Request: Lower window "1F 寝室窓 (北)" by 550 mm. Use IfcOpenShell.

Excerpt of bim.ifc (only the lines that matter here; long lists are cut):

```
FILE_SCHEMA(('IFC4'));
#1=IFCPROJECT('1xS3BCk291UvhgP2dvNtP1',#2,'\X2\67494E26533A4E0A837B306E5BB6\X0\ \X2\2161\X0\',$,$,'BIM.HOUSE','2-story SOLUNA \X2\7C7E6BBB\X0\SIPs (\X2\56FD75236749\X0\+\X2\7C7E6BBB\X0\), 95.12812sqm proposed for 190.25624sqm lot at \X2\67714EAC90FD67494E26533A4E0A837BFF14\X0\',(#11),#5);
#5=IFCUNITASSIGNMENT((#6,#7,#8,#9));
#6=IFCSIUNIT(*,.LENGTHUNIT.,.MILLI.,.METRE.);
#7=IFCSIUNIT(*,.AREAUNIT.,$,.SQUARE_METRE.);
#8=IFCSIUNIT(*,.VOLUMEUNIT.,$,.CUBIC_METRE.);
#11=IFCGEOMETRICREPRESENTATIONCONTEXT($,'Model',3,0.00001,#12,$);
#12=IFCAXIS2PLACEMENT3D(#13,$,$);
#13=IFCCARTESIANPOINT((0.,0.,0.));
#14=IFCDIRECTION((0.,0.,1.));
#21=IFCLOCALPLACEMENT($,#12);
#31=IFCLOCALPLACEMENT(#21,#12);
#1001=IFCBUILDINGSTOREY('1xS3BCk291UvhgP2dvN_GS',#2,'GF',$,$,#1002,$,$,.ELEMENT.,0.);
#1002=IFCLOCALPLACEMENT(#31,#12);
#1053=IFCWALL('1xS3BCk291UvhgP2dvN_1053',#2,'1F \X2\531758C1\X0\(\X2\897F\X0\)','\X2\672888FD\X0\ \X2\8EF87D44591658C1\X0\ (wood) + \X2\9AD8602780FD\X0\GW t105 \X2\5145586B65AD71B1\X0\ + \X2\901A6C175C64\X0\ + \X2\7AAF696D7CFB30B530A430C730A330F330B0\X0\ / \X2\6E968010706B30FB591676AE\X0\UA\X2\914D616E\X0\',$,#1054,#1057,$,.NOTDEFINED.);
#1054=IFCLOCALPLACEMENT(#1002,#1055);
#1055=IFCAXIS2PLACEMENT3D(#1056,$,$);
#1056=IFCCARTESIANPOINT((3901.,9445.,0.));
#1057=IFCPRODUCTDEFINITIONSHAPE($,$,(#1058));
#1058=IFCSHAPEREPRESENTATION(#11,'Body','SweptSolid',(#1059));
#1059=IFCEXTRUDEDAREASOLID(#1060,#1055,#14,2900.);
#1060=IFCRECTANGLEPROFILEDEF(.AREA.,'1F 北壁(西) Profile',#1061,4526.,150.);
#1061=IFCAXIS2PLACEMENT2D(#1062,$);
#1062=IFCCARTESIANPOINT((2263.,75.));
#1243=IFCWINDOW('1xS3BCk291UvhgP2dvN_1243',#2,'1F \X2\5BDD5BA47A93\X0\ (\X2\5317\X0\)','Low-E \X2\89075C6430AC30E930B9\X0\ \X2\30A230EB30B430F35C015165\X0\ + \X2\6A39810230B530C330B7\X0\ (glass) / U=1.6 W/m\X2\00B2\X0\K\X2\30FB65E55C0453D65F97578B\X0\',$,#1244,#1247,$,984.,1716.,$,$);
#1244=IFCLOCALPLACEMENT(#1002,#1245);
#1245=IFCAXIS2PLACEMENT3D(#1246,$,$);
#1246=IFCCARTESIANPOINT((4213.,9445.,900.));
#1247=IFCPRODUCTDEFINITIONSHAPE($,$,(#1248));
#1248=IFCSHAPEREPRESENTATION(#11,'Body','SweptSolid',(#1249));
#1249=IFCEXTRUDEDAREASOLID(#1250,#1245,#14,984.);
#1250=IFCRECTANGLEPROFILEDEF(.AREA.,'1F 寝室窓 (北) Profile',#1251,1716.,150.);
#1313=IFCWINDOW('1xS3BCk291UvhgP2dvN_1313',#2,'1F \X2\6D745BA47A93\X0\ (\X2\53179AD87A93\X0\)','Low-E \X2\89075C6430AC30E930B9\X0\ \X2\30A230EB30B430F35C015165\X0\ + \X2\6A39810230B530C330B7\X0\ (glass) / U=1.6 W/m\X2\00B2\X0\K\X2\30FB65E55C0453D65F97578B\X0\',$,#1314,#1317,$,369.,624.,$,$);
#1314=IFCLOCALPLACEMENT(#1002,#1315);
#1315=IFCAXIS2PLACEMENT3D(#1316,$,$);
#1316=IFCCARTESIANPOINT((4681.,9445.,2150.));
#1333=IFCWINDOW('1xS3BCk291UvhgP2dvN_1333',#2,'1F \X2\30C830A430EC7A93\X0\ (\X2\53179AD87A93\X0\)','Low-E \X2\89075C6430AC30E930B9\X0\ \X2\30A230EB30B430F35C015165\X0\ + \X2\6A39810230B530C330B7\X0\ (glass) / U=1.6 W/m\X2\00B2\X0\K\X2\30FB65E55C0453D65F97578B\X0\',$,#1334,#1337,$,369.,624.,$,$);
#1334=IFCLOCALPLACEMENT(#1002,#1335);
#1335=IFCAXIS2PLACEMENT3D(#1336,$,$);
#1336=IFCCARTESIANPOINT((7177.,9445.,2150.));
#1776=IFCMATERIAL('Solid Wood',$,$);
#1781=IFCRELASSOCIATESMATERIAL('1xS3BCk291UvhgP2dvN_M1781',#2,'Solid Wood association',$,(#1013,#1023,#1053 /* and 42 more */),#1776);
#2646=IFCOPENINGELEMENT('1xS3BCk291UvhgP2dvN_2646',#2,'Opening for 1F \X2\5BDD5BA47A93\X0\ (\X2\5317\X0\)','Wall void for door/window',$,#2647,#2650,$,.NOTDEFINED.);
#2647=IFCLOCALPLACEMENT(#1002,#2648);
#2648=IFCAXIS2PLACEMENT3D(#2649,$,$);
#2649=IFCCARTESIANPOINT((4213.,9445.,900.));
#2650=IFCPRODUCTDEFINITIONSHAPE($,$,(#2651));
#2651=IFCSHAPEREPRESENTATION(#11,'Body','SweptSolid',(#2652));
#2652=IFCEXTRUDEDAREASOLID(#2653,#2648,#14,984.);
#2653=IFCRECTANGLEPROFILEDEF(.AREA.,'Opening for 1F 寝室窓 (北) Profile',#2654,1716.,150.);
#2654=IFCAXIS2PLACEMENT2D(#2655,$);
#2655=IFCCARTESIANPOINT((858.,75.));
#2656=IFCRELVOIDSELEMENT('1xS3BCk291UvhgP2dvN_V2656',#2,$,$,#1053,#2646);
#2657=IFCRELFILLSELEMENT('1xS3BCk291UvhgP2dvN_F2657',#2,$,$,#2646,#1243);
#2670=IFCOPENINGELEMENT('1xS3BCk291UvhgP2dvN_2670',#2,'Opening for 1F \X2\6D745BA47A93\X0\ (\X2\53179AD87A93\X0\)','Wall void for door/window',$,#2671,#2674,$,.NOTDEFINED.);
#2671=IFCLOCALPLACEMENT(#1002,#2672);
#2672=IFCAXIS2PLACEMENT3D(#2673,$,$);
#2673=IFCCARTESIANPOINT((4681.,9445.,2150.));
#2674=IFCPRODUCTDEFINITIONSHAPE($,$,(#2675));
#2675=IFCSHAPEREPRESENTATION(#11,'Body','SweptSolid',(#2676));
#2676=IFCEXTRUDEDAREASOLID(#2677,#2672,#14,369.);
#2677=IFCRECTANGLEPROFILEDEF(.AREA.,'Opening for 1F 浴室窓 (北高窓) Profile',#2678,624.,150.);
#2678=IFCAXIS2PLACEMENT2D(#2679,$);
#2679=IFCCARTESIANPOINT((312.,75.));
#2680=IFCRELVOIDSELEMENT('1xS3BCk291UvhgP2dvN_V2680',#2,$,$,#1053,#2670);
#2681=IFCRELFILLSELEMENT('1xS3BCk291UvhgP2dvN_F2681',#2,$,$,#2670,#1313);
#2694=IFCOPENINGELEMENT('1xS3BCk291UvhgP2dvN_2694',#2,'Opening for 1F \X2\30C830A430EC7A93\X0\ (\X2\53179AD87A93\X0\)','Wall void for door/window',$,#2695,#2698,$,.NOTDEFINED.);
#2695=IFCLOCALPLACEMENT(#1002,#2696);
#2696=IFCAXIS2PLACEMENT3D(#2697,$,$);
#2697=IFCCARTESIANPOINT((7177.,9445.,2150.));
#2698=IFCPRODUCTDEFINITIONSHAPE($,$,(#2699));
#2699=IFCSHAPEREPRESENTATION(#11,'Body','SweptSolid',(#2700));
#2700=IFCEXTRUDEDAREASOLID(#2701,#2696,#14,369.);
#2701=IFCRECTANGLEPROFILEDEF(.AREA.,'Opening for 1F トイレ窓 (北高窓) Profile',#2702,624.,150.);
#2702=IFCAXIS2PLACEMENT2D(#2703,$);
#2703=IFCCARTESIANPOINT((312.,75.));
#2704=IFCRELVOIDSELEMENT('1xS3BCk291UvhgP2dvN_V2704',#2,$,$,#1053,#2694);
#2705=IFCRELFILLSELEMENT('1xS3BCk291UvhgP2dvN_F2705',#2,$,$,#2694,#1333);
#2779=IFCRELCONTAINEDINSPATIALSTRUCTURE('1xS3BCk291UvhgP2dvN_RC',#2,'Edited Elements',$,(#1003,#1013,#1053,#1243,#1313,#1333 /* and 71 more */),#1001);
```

```python
import numpy as np
import ifcopenshell
import ifcopenshell.api.geometry
import ifcopenshell.util.placement
import ifcopenshell.util.unit

model = ifcopenshell.open("bim.ifc")
unit_scale = ifcopenshell.util.unit.calculate_unit_scale(model)

window = model.by_guid("1xS3BCk291UvhgP2dvN_1243")
opening = window.FillsVoids[0].RelatingOpeningElement
dz = -0.55 / unit_scale

shift = np.array([0.0, 0.0, dz])
# The window is not placed relative to its opening, so move both.
for product in (opening, window):
    matrix = ifcopenshell.util.placement.get_local_placement(product.ObjectPlacement)
    matrix[:3, 3] += shift
    ifcopenshell.api.geometry.edit_object_placement(model, product=product, matrix=matrix, is_si=False)

print(f"moved by {dz * unit_scale:+.3f} m")

model.write("bim_edited.ifc")
```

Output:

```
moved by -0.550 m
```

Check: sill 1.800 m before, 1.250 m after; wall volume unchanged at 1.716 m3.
